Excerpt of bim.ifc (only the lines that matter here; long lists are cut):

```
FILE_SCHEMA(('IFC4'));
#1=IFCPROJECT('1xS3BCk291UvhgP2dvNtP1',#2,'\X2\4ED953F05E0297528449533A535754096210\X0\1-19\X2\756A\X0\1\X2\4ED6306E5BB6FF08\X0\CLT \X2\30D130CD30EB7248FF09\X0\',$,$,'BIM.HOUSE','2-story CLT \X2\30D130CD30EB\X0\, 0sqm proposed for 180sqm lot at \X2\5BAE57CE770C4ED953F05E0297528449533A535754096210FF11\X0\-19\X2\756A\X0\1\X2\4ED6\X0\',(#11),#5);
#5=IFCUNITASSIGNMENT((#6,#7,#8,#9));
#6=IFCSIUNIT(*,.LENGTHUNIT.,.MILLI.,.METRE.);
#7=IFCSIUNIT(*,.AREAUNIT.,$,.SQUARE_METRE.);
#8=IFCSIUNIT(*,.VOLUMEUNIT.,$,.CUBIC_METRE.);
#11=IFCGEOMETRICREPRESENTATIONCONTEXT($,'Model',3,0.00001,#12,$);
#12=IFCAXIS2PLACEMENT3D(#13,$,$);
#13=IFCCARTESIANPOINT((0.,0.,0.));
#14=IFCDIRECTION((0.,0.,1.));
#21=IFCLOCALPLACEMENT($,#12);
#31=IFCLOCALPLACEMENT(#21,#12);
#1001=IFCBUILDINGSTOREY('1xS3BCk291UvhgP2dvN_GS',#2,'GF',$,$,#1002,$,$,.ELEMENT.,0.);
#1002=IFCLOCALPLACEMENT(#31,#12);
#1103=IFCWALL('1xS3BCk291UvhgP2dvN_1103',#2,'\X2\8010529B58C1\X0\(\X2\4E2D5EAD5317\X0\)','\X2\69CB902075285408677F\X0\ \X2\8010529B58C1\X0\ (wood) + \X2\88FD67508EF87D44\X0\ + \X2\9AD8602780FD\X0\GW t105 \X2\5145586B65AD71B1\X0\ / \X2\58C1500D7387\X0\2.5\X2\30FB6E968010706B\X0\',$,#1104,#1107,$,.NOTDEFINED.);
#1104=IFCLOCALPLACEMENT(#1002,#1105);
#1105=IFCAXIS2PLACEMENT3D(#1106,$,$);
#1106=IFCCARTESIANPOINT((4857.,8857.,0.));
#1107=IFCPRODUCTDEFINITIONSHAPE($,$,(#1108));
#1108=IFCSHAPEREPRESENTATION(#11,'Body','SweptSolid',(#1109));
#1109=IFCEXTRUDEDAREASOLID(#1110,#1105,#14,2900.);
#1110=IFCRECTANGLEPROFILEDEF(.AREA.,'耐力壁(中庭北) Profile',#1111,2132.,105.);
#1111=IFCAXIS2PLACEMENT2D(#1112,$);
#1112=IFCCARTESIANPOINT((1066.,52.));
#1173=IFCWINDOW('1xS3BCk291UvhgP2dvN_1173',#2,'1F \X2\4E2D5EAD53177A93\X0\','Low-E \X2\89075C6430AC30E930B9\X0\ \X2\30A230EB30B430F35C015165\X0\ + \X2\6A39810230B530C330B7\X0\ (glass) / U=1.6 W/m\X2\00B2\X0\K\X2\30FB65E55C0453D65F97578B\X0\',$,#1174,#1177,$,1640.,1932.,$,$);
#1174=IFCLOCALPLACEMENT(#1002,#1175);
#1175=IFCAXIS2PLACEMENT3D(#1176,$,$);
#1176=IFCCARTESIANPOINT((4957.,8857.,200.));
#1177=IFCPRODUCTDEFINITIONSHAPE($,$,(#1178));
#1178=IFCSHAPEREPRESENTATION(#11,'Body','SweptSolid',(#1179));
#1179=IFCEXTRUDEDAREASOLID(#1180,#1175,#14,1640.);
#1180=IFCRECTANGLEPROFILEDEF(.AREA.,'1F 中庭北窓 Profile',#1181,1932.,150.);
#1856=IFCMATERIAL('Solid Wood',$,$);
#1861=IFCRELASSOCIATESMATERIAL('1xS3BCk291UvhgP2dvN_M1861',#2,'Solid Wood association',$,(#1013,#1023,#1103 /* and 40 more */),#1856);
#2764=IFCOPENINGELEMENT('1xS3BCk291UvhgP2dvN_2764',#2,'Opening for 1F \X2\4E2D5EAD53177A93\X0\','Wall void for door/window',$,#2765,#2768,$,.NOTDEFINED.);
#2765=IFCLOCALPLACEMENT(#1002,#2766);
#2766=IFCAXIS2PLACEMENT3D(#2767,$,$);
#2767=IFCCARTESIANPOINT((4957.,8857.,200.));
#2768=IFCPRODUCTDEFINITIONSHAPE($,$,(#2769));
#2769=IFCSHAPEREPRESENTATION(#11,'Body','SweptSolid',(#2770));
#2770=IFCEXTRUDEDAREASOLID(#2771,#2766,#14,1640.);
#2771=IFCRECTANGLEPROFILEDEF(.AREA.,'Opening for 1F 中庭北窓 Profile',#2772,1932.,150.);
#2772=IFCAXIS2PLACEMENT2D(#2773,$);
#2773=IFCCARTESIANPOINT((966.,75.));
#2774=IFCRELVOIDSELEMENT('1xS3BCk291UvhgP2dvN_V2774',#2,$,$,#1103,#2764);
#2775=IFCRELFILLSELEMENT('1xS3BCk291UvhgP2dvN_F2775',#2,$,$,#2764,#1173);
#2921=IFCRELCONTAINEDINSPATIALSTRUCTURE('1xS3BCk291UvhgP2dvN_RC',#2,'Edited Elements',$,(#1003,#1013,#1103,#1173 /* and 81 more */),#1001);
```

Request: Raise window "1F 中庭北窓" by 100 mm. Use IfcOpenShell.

```python
import numpy as np
import ifcopenshell
import ifcopenshell.api.geometry
import ifcopenshell.util.placement
import ifcopenshell.util.unit

model = ifcopenshell.open("bim.ifc")
unit_scale = ifcopenshell.util.unit.calculate_unit_scale(model)

window = model.by_guid("1xS3BCk291UvhgP2dvN_1173")
opening = window.FillsVoids[0].RelatingOpeningElement
dz = 100.0

shift = np.array([0.0, 0.0, dz])
# The window is not placed relative to its opening, so move both.
for product in (opening, window):
    matrix = ifcopenshell.util.placement.get_local_placement(product.ObjectPlacement)
    matrix[:3, 3] += shift
    ifcopenshell.api.geometry.edit_object_placement(model, product=product, matrix=matrix, is_si=False)

print(f"moved by {dz * unit_scale:+.3f} m")

model.write("bim_rev.ifc")
```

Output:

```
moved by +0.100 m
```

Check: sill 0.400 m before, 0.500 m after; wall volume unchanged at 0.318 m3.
